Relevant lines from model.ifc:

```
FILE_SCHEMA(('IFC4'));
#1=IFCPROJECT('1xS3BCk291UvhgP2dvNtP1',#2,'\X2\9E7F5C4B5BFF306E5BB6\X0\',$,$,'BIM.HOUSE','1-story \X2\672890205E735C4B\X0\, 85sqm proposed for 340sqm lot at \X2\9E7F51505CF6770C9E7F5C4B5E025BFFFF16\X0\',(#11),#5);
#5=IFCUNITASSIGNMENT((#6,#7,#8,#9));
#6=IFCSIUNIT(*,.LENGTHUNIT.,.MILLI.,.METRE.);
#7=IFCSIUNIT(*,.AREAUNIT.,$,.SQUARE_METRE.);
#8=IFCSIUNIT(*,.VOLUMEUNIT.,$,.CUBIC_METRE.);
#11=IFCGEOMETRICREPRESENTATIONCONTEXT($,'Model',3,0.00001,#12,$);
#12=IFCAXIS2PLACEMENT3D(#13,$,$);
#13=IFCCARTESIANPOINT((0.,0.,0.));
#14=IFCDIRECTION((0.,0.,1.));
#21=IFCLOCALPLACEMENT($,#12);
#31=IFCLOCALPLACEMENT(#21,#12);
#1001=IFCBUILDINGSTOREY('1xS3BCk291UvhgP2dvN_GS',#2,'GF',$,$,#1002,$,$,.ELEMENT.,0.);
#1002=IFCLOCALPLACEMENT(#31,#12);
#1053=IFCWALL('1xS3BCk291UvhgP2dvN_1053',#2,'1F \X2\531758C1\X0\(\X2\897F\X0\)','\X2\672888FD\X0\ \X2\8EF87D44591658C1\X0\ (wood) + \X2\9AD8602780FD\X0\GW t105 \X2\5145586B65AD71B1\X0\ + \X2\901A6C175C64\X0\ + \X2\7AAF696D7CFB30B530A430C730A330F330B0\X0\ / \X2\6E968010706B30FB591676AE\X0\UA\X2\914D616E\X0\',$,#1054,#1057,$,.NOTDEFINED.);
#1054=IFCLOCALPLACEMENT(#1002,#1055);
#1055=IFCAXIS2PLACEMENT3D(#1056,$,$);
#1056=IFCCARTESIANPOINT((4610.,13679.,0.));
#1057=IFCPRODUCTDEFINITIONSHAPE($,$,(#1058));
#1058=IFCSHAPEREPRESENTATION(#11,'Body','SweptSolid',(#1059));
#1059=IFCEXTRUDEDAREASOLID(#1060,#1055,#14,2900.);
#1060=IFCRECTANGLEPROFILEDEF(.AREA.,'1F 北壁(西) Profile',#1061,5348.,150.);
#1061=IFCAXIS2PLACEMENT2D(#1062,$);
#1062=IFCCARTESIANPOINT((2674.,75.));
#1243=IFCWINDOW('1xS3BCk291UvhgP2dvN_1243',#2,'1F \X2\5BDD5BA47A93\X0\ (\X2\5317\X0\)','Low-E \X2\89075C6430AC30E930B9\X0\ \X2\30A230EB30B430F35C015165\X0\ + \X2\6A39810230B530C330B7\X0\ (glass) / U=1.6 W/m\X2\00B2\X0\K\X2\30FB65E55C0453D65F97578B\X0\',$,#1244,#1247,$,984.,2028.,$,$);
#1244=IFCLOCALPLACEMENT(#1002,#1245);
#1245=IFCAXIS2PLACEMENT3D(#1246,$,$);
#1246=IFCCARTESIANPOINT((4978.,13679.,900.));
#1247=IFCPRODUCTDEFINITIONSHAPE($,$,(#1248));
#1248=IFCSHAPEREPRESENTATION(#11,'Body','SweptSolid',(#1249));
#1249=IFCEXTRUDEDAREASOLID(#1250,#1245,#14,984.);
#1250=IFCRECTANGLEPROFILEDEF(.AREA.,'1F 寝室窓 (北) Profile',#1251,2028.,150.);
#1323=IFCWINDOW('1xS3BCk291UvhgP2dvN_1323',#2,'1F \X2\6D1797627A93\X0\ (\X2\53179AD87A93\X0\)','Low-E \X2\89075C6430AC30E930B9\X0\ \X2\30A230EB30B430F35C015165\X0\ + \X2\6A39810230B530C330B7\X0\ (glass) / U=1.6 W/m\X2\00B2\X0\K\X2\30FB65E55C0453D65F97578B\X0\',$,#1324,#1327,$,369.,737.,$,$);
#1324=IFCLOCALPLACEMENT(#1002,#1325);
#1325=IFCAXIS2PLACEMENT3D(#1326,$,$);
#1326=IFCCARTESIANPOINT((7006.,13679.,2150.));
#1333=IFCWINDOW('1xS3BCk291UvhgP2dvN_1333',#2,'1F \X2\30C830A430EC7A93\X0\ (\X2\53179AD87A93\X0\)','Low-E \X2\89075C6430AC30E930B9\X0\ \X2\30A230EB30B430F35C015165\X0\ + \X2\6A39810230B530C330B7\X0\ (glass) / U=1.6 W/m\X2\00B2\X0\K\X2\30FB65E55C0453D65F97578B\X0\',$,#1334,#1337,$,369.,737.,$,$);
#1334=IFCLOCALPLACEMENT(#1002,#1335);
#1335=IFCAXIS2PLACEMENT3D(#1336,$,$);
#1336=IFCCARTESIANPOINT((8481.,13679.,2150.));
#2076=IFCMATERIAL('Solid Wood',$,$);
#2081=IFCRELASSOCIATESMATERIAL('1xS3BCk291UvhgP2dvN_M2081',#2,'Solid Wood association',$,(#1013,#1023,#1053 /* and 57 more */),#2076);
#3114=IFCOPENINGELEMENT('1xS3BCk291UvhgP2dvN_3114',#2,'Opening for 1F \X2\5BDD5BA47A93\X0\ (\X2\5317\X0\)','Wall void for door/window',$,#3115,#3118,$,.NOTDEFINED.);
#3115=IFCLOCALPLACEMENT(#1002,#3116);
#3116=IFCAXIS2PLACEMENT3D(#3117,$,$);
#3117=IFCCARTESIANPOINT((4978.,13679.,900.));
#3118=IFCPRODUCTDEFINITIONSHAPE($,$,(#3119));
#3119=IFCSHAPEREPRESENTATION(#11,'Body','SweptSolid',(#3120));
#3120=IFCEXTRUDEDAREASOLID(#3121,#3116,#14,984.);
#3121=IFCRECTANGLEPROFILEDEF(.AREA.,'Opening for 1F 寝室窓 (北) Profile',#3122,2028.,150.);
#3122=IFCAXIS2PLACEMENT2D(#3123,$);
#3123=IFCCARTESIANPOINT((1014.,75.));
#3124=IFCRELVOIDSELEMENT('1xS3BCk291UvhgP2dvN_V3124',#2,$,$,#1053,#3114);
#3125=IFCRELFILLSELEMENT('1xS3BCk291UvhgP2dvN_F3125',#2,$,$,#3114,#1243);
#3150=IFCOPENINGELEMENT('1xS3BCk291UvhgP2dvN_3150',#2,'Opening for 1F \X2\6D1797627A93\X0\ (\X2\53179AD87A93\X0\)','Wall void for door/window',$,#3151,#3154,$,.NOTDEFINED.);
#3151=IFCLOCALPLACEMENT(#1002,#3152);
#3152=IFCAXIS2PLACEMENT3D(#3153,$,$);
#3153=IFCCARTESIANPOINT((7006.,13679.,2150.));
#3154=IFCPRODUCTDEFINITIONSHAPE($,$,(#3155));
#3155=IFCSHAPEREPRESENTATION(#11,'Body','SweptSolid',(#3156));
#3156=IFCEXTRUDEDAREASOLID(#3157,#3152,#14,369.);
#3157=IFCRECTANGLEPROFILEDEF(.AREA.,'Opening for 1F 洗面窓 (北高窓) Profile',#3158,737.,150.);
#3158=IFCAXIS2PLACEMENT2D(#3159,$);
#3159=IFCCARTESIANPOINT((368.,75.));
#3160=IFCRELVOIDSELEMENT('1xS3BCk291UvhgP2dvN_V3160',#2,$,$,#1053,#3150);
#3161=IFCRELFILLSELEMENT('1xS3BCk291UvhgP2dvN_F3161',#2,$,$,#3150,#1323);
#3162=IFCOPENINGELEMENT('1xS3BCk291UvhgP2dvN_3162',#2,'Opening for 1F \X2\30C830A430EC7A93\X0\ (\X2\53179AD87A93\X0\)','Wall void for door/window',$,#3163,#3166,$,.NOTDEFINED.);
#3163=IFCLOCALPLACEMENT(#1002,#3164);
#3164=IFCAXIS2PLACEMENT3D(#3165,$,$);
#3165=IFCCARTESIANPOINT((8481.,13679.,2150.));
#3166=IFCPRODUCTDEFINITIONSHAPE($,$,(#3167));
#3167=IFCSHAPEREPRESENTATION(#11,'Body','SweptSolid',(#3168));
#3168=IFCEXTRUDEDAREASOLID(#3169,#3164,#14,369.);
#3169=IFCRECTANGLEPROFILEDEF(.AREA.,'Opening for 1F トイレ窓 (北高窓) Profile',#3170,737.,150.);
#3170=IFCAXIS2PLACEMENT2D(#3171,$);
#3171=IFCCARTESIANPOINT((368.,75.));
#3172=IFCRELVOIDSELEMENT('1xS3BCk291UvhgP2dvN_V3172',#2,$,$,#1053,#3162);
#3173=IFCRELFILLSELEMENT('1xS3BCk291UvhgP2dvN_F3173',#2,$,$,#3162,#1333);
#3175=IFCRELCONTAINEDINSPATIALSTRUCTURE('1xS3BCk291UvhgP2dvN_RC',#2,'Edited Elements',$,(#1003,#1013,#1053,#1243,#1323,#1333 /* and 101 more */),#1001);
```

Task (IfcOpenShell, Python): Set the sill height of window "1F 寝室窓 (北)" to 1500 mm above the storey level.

```python
import numpy as np
import ifcopenshell
import ifcopenshell.api.geometry
import ifcopenshell.geom
import ifcopenshell.util.element
import ifcopenshell.util.placement
import ifcopenshell.util.shape
import ifcopenshell.util.unit

model = ifcopenshell.open("model.ifc")
unit_scale = ifcopenshell.util.unit.calculate_unit_scale(model)

window = model.by_id(1243)
opening = window.FillsVoids[0].RelatingOpeningElement
storey = ifcopenshell.util.element.get_container(window, ifc_class="IfcBuildingStorey")
level = ifcopenshell.util.placement.get_local_placement(storey.ObjectPlacement)[2, 3]

# The opening's origin need not be at the sill, so measure its lowest point.
shape = ifcopenshell.geom.create_shape(ifcopenshell.geom.settings(), opening)
bottom = ifcopenshell.util.shape.get_shape_bottom_elevation(shape, shape.geometry) / unit_scale
dz = level + 1500.0 - bottom

shift = np.array([0.0, 0.0, dz])
# The window is not placed relative to its opening, so move both.
for product in (opening, window):
    matrix = ifcopenshell.util.placement.get_local_placement(product.ObjectPlacement)
    matrix[:3, 3] += shift
    ifcopenshell.api.geometry.edit_object_placement(model, product=product, matrix=matrix, is_si=False)

print(f"moved by {dz * unit_scale:+.3f} m")

model.write("model_rev.ifc")
```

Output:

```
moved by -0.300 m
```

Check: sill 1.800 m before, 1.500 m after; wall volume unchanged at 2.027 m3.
